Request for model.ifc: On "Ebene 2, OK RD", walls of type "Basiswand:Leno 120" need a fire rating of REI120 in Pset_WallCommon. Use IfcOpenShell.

First a look at what the model holds.

```python
import ifcopenshell
import ifcopenshell.util.element

model = ifcopenshell.open("model.ifc")
print(model.schema)
storey = next(s for s in model.by_type("IfcBuildingStorey") if s.Name == "Ebene 2, OK RD")
walls = [e for e in ifcopenshell.util.element.get_decomposition(storey) if e.is_a("IfcWall")]
seen = {}
for e in walls:
    element_type = ifcopenshell.util.element.get_type(e)
    key = (element_type.Name if element_type != e and element_type else None, ifcopenshell.util.element.get_pset(e, "Pset_WallCommon", "FireRating"))
    seen[key] = seen.get(key, 0) + 1
for (name, value), count in sorted(seen.items(), key=str):
    print(count, "x", name, "|", value)
```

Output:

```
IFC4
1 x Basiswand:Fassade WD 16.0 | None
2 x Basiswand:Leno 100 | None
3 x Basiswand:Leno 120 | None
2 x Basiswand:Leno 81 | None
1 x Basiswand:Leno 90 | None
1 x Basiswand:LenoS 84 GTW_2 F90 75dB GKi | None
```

```python
import ifcopenshell
import ifcopenshell.api.pset
import ifcopenshell.util.element

model = ifcopenshell.open("model.ifc")

storey = next(s for s in model.by_type("IfcBuildingStorey") if s.Name == "Ebene 2, OK RD")
walls = [e for e in ifcopenshell.util.element.get_decomposition(storey) if e.is_a("IfcWall")]

count = 0
for e in walls:
    element_type = ifcopenshell.util.element.get_type(e)
    if element_type in (None, e) or element_type.Name != "Basiswand:Leno 120":
        continue
    # add_pset returns the element's existing set when there is one.
    pset = ifcopenshell.api.pset.add_pset(model, product=e, name="Pset_WallCommon")
    ifcopenshell.api.pset.edit_pset(model, pset=pset, properties={"FireRating": "REI120"})
    count += 1

print(count, "walls updated")

model.write("model_edited.ifc")
```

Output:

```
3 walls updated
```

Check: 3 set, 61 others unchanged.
